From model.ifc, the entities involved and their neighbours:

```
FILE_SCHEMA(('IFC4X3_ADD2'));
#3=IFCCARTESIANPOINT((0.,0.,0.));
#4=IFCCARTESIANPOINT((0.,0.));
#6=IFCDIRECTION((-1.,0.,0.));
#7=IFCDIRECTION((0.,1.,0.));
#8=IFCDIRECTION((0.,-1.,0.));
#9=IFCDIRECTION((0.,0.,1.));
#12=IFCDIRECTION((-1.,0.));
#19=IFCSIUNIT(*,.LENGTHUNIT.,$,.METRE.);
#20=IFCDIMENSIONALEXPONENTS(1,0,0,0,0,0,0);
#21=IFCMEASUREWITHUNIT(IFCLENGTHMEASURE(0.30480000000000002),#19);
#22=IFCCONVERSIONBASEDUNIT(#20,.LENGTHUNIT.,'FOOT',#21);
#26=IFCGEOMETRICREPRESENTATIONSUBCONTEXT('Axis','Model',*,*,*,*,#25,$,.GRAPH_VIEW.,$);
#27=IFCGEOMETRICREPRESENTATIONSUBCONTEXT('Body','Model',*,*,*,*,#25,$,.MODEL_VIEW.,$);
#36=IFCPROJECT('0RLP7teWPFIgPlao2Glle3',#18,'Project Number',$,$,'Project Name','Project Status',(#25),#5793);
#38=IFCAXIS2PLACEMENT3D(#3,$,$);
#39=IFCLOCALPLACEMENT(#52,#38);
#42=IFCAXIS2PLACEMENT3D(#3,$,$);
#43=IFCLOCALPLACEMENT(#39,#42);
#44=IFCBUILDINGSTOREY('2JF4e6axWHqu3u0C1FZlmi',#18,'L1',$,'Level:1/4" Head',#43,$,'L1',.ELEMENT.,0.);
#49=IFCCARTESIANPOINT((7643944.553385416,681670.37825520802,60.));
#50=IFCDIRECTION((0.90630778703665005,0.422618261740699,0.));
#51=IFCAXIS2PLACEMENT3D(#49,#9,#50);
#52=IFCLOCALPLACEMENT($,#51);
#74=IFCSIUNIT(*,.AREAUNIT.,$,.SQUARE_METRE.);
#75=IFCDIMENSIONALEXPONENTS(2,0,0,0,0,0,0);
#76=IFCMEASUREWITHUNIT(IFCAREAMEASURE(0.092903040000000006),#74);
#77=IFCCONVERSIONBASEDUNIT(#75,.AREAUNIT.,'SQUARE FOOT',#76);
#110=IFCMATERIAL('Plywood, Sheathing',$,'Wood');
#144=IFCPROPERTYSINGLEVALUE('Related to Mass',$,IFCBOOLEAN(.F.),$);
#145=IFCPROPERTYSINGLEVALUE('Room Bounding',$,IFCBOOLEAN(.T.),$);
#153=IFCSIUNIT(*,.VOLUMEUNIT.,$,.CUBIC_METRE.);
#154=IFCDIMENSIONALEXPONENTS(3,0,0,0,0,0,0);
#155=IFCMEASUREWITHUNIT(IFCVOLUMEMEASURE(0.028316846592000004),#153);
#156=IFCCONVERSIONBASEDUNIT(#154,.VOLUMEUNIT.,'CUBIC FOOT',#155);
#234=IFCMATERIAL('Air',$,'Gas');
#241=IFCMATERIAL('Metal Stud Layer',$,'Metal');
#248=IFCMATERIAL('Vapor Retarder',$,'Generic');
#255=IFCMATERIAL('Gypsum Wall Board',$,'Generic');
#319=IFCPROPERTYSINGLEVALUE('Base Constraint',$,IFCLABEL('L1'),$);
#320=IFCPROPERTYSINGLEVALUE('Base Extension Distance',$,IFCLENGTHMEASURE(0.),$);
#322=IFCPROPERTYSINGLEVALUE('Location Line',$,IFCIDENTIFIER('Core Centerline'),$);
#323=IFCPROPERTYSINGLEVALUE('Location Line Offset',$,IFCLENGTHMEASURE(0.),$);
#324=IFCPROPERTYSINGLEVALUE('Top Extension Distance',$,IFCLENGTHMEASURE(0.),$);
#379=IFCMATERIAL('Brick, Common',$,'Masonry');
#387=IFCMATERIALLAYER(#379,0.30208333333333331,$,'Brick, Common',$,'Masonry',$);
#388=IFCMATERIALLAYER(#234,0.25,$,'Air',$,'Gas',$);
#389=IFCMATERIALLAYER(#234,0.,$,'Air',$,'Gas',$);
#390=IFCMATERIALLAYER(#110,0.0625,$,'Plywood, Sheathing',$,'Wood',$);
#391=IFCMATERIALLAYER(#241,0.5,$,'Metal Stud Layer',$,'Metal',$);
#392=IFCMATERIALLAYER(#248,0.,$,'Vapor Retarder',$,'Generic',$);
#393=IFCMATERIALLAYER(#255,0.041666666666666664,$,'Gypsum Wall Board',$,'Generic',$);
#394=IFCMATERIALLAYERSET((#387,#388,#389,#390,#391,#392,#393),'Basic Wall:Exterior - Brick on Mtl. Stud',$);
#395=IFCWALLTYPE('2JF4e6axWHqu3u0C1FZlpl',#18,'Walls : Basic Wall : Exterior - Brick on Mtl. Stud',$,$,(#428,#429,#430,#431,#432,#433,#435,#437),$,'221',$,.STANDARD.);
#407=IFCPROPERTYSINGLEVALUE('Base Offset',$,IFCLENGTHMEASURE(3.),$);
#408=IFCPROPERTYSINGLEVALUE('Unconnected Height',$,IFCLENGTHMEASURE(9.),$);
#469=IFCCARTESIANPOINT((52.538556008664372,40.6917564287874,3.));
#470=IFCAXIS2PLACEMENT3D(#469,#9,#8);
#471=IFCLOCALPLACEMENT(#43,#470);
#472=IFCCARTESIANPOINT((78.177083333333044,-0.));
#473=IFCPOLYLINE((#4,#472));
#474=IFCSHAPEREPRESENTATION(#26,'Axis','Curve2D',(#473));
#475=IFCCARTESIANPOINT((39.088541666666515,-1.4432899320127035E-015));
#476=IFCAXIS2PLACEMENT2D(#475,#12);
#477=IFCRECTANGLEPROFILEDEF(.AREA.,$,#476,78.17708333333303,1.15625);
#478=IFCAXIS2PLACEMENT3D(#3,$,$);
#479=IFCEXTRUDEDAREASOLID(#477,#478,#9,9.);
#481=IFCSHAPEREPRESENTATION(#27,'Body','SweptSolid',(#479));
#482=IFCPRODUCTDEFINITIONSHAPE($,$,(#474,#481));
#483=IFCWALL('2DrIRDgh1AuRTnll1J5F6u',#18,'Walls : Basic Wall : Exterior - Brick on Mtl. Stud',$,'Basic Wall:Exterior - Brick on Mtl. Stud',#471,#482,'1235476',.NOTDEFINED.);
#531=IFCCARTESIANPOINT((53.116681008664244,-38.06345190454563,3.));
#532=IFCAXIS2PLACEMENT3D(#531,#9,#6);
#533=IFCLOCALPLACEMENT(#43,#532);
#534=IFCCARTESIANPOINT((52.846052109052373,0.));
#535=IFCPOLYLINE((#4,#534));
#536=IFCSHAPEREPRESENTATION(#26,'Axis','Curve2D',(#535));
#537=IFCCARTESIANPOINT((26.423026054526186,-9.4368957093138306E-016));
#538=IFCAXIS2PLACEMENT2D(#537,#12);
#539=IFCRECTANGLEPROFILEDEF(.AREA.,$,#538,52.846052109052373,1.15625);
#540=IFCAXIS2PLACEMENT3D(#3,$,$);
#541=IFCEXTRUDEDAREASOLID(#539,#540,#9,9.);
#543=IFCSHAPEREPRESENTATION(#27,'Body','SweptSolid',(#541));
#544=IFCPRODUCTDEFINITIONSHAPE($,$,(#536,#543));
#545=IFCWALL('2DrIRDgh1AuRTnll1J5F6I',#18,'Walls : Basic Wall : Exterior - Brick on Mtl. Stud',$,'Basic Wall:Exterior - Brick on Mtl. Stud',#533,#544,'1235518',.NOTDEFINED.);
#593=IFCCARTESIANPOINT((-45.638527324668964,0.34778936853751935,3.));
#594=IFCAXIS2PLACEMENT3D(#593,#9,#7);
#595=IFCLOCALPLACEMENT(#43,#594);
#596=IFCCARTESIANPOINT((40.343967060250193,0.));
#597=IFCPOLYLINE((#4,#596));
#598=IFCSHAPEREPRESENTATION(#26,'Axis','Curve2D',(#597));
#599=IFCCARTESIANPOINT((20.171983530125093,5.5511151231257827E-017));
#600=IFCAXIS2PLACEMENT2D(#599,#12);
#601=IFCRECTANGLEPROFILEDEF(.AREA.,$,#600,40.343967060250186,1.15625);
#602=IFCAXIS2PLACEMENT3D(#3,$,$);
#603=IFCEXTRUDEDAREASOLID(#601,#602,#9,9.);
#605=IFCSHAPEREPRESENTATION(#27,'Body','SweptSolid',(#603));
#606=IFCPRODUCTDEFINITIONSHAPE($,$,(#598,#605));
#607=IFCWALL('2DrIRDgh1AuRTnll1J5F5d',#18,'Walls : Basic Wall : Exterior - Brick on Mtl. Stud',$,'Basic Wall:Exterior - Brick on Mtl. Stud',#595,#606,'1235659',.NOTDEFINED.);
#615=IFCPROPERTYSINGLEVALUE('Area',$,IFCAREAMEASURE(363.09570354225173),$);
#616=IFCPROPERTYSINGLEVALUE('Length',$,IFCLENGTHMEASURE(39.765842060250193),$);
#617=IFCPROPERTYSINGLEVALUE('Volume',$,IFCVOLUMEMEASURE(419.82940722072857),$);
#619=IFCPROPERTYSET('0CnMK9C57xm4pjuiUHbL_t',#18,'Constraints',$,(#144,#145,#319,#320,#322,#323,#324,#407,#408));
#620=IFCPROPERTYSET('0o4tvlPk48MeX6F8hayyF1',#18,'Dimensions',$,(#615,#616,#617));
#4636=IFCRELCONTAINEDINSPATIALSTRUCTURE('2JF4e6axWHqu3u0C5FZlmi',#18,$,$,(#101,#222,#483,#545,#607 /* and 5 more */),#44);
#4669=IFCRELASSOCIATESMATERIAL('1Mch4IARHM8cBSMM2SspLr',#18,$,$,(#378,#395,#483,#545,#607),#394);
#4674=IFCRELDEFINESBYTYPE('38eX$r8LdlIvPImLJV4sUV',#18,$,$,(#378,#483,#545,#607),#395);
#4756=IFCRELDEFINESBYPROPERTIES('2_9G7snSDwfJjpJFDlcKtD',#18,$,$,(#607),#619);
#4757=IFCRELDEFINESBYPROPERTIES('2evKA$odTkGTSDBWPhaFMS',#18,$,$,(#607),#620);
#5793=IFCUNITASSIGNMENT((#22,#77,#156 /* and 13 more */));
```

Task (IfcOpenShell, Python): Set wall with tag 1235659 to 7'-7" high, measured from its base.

```python
import ifcopenshell
import ifcopenshell.api.pset
import ifcopenshell.geom
import ifcopenshell.util.element
import ifcopenshell.util.representation
import ifcopenshell.util.shape
import ifcopenshell.util.unit

model = ifcopenshell.open("model.ifc")
unit_scale = ifcopenshell.util.unit.calculate_unit_scale(model)
area_scale = ifcopenshell.util.unit.calculate_unit_scale(model, "AREAUNIT")
volume_scale = ifcopenshell.util.unit.calculate_unit_scale(model, "VOLUMEUNIT")
settings = ifcopenshell.geom.settings()


def volume(element):
    """Net volume in cubic metres, openings subtracted."""
    shape = ifcopenshell.geom.create_shape(settings, element)
    return ifcopenshell.util.shape.get_volume(shape.geometry)


wall = model.by_id(607)
before = volume(wall)

body = ifcopenshell.util.representation.get_representation(wall, "Model", "Body")
solid = body.Items[0]
old_height = solid.Depth
solid.Depth = 91 * 0.0254 / unit_scale
after = volume(wall)
thickness = 0.3524  # wall thickness in metres

# Update the stored height, areas and volumes.
pset = model.by_id(ifcopenshell.util.element.get_pset(wall, "Constraints", should_inherit=False)["id"])
ifcopenshell.api.pset.edit_pset(model, pset=pset, properties={
    "Unconnected Height": model.create_entity("IfcLengthMeasure", solid.Depth),
})
pset = model.by_id(ifcopenshell.util.element.get_pset(wall, "Dimensions", should_inherit=False)["id"])
ifcopenshell.api.pset.edit_pset(model, pset=pset, properties={
    "Area": model.create_entity("IfcAreaMeasure", after / thickness / area_scale),
    "Volume": model.create_entity("IfcVolumeMeasure", after / volume_scale),
})

print(f"height {old_height:g} -> {solid.Depth:g}, volume {before:.3f} -> {after:.3f} m3")

model.write("model_rev.ifc")
```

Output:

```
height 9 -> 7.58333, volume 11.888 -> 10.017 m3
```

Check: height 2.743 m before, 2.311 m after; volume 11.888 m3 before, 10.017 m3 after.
